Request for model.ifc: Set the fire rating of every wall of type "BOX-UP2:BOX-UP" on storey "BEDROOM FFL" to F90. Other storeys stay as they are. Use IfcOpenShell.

First a look at what the model holds.

```python
import ifcopenshell
import ifcopenshell.util.element

model = ifcopenshell.open("model.ifc")
print(model.schema)
storey = next(s for s in model.by_type("IfcBuildingStorey") if s.Name == "BEDROOM FFL")
walls = [e for e in ifcopenshell.util.element.get_decomposition(storey) if e.is_a("IfcWall")]
seen = {}
for e in walls:
    element_type = ifcopenshell.util.element.get_type(e)
    key = (element_type.Name if element_type != e and element_type else None, ifcopenshell.util.element.get_pset(e, "Pset_WallCommon", "FireRating"))
    seen[key] = seen.get(key, 0) + 1
for (name, value), count in sorted(seen.items(), key=str):
    print(count, "x", name, "|", value)
```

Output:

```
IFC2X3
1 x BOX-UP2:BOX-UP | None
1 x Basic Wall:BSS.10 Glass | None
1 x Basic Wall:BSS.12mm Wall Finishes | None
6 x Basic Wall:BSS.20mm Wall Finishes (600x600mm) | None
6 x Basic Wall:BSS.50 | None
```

```python
import ifcopenshell
import ifcopenshell.api.pset
import ifcopenshell.util.element

model = ifcopenshell.open("model.ifc")

storey = next(s for s in model.by_type("IfcBuildingStorey") if s.Name == "BEDROOM FFL")
walls = [e for e in ifcopenshell.util.element.get_decomposition(storey) if e.is_a("IfcWall")]

count = 0
for e in walls:
    element_type = ifcopenshell.util.element.get_type(e)
    if element_type in (None, e) or element_type.Name != "BOX-UP2:BOX-UP":
        continue
    # add_pset returns the element's existing set when there is one.
    pset = ifcopenshell.api.pset.add_pset(model, product=e, name="Pset_WallCommon")
    ifcopenshell.api.pset.edit_pset(model, pset=pset, properties={"FireRating": "F90"})
    count += 1

print(count, "walls updated")

model.write("model_v2.ifc")
```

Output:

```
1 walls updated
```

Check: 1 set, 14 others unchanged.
